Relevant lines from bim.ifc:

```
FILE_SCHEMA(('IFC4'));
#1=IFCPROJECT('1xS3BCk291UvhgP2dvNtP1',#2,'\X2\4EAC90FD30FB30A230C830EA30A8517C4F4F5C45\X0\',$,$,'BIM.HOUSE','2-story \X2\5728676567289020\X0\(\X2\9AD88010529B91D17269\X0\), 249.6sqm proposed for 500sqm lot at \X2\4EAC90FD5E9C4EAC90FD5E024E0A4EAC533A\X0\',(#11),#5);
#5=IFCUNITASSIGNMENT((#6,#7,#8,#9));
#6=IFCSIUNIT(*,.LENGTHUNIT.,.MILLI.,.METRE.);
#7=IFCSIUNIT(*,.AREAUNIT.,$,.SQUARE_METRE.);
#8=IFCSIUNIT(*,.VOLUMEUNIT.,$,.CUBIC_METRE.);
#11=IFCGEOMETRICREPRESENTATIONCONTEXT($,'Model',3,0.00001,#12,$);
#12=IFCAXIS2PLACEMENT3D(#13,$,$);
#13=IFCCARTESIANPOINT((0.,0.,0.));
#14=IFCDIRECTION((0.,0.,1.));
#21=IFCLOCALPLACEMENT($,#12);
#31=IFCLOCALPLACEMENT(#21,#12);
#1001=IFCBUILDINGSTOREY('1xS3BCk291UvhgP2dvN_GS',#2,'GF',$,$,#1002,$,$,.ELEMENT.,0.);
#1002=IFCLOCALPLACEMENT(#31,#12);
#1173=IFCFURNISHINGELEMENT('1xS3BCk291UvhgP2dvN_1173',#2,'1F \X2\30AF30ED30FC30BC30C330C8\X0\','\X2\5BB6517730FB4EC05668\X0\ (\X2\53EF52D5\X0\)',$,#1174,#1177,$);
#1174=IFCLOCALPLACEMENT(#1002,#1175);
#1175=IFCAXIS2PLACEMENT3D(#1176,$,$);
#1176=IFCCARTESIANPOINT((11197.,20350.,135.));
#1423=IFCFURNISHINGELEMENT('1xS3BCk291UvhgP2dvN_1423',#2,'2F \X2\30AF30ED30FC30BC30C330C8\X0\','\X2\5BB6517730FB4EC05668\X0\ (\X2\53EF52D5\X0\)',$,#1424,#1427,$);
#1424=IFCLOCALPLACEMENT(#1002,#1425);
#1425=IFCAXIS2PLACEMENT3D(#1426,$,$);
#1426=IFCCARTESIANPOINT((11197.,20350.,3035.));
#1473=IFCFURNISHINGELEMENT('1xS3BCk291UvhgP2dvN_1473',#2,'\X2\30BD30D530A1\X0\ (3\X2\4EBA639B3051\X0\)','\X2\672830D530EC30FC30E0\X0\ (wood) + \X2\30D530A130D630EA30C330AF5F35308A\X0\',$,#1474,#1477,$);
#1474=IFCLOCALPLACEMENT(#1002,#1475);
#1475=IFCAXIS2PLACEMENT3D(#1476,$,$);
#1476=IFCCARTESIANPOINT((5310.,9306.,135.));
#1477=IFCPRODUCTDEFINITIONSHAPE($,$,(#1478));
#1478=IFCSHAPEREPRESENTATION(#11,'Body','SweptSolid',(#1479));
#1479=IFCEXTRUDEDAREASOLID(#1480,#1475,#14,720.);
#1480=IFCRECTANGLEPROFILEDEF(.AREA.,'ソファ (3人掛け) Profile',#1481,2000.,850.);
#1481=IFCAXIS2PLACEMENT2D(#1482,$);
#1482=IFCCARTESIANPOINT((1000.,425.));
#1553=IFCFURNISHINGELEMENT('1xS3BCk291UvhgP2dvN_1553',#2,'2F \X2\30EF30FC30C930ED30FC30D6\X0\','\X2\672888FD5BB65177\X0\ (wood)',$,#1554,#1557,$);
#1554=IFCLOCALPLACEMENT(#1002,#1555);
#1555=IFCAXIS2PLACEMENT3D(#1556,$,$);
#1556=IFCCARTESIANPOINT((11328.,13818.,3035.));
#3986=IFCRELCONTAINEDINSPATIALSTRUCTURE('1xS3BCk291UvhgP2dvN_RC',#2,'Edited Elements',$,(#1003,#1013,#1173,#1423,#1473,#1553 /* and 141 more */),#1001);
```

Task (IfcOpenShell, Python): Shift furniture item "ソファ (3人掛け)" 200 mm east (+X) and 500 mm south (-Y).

```python
import ifcopenshell
import ifcopenshell.api.geometry
import ifcopenshell.util.placement
import ifcopenshell.util.unit

model = ifcopenshell.open("bim.ifc")
unit_scale = ifcopenshell.util.unit.calculate_unit_scale(model)

item = model.by_id(1473)
matrix = ifcopenshell.util.placement.get_local_placement(item.ObjectPlacement)
matrix[0, 3] += 0.2 / unit_scale
matrix[1, 3] -= 0.5 / unit_scale
ifcopenshell.api.geometry.edit_object_placement(model, product=item, matrix=matrix, is_si=False)

print(ifcopenshell.util.placement.get_local_placement(item.ObjectPlacement).round(3) + 0.0)

model.write("bim_v2.ifc")
```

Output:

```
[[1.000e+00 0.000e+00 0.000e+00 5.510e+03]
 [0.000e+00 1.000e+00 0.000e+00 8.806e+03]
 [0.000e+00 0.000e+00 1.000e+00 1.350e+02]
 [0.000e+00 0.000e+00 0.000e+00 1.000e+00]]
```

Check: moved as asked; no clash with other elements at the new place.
